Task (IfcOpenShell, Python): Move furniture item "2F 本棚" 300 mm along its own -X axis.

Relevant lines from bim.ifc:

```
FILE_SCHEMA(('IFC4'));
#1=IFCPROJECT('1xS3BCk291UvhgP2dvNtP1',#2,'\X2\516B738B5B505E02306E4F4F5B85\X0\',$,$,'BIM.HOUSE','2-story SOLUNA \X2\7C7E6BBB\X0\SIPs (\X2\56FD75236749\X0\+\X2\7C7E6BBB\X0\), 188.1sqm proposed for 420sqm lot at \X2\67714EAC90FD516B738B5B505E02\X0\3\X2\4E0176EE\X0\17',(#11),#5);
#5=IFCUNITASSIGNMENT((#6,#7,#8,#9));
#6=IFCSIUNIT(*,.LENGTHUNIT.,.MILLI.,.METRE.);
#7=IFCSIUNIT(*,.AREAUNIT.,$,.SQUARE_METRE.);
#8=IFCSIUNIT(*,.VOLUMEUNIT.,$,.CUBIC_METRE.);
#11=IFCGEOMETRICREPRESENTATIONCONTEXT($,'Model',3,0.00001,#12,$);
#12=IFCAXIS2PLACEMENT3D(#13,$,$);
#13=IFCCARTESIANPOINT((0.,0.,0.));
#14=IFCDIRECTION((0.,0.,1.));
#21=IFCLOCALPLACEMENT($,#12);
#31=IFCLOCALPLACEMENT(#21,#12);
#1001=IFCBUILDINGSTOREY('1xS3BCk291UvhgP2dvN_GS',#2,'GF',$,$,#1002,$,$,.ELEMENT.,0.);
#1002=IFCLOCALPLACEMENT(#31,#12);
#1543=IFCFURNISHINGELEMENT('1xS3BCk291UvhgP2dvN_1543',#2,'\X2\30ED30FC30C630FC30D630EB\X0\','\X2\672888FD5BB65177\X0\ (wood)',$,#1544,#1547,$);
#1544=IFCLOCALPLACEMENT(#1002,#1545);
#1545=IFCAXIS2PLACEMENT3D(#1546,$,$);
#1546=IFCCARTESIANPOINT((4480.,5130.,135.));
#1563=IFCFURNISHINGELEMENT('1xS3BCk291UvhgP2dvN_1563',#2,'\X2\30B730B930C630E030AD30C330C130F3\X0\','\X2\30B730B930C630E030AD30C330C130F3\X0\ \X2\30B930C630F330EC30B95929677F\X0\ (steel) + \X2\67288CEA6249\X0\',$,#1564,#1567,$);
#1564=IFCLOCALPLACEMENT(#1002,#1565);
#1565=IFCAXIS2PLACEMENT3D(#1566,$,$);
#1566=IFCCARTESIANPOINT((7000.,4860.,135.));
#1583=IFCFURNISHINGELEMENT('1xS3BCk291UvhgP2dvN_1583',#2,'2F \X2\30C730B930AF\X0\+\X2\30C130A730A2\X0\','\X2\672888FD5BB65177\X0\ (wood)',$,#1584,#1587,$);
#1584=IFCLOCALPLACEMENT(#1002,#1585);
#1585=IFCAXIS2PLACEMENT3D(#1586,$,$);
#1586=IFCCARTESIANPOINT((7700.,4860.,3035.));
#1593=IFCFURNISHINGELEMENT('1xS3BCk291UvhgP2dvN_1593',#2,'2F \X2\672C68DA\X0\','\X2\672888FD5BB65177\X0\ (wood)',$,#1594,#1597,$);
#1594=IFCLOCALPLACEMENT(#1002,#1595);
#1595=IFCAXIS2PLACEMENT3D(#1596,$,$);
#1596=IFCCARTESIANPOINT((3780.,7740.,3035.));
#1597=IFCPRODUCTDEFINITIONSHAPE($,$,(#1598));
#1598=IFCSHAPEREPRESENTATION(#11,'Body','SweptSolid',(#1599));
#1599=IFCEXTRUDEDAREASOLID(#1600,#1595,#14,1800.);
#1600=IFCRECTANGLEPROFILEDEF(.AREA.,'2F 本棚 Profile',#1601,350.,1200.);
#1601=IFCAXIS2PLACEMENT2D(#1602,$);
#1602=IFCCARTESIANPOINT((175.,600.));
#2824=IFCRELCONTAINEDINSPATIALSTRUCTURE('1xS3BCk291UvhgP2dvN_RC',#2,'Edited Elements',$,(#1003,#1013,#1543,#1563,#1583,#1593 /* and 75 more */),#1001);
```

```python
import ifcopenshell
import ifcopenshell.api.geometry
import ifcopenshell.util.placement
import ifcopenshell.util.unit

model = ifcopenshell.open("bim.ifc")
unit_scale = ifcopenshell.util.unit.calculate_unit_scale(model)

item = model.by_id(1593)
matrix = ifcopenshell.util.placement.get_local_placement(item.ObjectPlacement)
matrix[:3, 3] -= matrix[:3, 0] * 0.3 / unit_scale
ifcopenshell.api.geometry.edit_object_placement(model, product=item, matrix=matrix, is_si=False)

print(ifcopenshell.util.placement.get_local_placement(item.ObjectPlacement).round(3) + 0.0)

model.write("bim_edited.ifc")
```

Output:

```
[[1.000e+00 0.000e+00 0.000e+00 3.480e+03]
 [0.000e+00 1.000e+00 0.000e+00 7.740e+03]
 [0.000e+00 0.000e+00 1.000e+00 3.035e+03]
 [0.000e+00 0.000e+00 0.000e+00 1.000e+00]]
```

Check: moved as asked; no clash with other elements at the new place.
